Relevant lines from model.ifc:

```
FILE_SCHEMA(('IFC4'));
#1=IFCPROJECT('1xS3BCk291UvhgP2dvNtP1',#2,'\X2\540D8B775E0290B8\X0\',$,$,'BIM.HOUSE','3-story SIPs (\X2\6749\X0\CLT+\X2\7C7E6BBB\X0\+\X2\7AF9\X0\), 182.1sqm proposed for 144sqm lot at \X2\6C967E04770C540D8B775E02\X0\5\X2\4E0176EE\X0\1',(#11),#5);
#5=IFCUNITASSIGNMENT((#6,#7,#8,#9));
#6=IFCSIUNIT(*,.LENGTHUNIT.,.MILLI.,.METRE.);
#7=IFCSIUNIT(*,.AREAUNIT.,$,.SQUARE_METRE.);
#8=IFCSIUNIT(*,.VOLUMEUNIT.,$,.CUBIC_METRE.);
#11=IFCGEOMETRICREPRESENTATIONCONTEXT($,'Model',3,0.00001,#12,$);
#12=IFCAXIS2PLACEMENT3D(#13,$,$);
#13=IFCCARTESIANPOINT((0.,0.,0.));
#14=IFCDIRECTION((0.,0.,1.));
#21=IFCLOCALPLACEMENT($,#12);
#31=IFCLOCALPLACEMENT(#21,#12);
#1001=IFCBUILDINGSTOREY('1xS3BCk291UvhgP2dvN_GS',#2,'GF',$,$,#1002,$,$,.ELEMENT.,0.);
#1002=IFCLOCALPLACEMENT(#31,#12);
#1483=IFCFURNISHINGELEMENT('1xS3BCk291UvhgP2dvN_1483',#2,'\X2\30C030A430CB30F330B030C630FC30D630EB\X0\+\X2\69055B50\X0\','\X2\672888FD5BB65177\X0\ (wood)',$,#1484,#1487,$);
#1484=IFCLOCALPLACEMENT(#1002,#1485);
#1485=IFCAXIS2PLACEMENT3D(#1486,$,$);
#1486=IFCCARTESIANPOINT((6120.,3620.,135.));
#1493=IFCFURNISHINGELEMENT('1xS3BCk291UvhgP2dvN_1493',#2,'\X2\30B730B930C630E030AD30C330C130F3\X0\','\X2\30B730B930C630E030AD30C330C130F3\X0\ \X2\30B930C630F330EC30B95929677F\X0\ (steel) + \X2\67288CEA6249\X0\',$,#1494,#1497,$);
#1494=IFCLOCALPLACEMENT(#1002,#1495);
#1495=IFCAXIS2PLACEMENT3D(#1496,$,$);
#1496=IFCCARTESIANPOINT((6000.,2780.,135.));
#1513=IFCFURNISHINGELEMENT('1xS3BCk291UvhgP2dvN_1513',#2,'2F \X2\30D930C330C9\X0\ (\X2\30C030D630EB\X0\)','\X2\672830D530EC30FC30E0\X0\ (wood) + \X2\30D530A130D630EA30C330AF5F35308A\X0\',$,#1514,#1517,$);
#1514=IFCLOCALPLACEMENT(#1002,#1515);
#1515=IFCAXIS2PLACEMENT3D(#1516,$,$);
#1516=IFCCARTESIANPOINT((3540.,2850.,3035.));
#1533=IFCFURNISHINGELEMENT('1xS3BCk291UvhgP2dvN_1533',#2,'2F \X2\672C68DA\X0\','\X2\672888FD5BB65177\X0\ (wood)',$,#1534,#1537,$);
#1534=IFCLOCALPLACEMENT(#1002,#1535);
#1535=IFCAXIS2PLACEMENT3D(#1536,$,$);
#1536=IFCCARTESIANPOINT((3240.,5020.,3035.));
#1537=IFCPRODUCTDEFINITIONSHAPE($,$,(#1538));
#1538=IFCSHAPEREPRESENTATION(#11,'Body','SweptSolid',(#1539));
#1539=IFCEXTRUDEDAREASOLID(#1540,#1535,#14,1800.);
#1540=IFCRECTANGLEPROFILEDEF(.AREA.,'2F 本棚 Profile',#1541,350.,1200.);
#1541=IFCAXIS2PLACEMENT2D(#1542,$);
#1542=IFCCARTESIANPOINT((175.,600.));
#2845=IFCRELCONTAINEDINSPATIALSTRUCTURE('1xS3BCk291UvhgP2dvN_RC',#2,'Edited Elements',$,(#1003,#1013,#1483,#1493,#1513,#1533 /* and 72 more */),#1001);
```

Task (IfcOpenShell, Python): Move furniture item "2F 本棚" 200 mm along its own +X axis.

```python
import ifcopenshell
import ifcopenshell.api.geometry
import ifcopenshell.util.placement

model = ifcopenshell.open("model.ifc")

item = model.by_id(1533)
matrix = ifcopenshell.util.placement.get_local_placement(item.ObjectPlacement)
matrix[:3, 3] += matrix[:3, 0] * 200.0
ifcopenshell.api.geometry.edit_object_placement(model, product=item, matrix=matrix, is_si=False)

print(ifcopenshell.util.placement.get_local_placement(item.ObjectPlacement).round(3) + 0.0)

model.write("model_v2.ifc")
```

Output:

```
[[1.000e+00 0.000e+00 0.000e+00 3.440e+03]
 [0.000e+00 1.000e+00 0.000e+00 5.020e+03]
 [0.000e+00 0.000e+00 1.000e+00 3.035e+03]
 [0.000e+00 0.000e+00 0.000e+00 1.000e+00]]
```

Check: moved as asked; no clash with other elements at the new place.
